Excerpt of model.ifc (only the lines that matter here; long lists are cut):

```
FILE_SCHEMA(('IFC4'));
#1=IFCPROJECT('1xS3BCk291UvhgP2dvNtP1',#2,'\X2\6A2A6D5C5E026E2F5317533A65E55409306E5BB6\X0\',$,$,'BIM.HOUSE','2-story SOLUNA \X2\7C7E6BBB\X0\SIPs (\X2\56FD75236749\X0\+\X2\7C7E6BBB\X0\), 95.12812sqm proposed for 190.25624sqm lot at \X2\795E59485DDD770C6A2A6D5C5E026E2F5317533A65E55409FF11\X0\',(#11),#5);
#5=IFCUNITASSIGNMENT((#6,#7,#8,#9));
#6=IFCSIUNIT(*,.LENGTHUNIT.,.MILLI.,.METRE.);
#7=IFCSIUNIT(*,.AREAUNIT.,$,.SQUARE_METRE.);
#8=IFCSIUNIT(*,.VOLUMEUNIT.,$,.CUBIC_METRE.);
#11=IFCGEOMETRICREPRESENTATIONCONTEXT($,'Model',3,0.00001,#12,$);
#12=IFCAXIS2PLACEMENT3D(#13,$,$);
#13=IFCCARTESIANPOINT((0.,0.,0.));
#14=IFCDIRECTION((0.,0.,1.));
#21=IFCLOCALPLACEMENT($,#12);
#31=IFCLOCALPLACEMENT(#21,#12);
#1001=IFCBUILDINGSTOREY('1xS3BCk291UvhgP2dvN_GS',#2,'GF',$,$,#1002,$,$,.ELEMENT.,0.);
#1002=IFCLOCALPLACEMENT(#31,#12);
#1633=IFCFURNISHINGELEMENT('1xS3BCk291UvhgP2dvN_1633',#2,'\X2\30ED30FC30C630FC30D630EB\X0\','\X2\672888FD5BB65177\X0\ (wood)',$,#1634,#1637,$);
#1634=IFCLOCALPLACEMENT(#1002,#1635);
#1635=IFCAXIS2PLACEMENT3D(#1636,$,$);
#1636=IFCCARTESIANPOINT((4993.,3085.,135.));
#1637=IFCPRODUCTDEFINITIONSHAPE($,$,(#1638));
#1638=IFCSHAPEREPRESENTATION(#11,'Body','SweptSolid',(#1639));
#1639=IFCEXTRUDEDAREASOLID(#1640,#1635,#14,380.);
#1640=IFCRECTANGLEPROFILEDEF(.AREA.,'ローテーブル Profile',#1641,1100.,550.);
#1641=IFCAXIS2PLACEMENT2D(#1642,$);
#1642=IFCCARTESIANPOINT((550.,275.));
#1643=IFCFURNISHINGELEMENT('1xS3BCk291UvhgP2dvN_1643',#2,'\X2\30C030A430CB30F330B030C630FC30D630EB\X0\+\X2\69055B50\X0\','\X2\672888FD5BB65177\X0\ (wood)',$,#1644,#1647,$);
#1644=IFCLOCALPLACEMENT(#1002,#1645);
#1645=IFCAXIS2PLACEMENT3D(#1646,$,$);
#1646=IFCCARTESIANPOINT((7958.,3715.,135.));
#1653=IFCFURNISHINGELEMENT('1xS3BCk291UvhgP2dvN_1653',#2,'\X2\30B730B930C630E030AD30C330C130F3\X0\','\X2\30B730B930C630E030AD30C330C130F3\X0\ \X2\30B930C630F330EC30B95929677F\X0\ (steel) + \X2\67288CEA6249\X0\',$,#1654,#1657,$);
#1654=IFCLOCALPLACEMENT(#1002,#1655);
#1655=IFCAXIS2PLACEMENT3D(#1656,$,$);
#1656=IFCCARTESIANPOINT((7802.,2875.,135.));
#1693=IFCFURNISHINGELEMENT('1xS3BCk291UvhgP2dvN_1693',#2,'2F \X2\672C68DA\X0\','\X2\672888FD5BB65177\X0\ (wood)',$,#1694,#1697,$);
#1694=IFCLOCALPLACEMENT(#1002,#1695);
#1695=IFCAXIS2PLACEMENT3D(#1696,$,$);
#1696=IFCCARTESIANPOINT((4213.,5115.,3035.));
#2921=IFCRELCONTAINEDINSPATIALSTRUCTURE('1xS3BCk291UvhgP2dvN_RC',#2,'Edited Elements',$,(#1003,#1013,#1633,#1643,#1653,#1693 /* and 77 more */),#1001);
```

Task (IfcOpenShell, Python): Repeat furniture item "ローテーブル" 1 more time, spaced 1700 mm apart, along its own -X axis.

```python
import ifcopenshell
import ifcopenshell.api.geometry
import ifcopenshell.api.root
import ifcopenshell.util.element
import ifcopenshell.util.placement
import ifcopenshell.util.unit

model = ifcopenshell.open("model.ifc")
unit_scale = ifcopenshell.util.unit.calculate_unit_scale(model)


def reuse_history(source, copy):
    """copy_class also copies each property set's owner history, people and application; keep the originals."""
    for rel in copy.IsDefinedBy:
        if rel.is_a("IfcRelDefinesByProperties") and (history := rel.RelatingPropertyDefinition.OwnerHistory):
            rel.RelatingPropertyDefinition.OwnerHistory = source.OwnerHistory
            ifcopenshell.util.element.remove_deep2(model, history)


source = model.by_guid("1xS3BCk291UvhgP2dvN_1633")
base = ifcopenshell.util.placement.get_local_placement(source.ObjectPlacement)
step = -base[:3, 0] * 1.7 / unit_scale

for i in range(1, 2):
    copy = ifcopenshell.api.root.copy_class(model, product=source)
    copy.Representation = ifcopenshell.util.element.copy_deep(
        model, source.Representation, exclude=["IfcGeometricRepresentationContext", "IfcRepresentationMap"]
    )
    reuse_history(source, copy)
    matrix = base.copy()
    matrix[:3, 3] += i * step
    print("added at", matrix[:3, 3].round(3) + 0.0)
    ifcopenshell.api.geometry.edit_object_placement(model, product=copy, matrix=matrix, is_si=False)

model.write("model_v2.ifc")
```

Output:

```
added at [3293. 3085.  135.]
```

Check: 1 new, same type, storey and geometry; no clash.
